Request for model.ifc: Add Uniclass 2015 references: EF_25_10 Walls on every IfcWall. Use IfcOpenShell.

First a look at what the model holds.

```python
import ifcopenshell

model = ifcopenshell.open("model.ifc")
print(model.schema)
print("classifications:", [c.Name for c in model.by_type("IfcClassification")])
for ifc_class in ("IfcDoor", "IfcRoof", "IfcStair", "IfcWall", "IfcWindow"):
    print(ifc_class, len(model.by_type(ifc_class)))
```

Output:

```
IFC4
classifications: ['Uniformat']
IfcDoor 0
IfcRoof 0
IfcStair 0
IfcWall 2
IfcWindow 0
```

```python
import ifcopenshell
import ifcopenshell.api.classification

model = ifcopenshell.open("model.ifc")

system = ifcopenshell.api.classification.add_classification(model, classification="Uniclass 2015")

codes = {
    "IfcWall": ("EF_25_10", "Walls"),
}
for ifc_class, (code, name) in codes.items():
    products = model.by_type(ifc_class)
    ifcopenshell.api.classification.add_reference(
        model, products=products, classification=system, identification=code, name=name
    )
    print(code, len(products))

model.write("model-out.ifc")
```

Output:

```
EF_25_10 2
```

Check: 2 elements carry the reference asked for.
